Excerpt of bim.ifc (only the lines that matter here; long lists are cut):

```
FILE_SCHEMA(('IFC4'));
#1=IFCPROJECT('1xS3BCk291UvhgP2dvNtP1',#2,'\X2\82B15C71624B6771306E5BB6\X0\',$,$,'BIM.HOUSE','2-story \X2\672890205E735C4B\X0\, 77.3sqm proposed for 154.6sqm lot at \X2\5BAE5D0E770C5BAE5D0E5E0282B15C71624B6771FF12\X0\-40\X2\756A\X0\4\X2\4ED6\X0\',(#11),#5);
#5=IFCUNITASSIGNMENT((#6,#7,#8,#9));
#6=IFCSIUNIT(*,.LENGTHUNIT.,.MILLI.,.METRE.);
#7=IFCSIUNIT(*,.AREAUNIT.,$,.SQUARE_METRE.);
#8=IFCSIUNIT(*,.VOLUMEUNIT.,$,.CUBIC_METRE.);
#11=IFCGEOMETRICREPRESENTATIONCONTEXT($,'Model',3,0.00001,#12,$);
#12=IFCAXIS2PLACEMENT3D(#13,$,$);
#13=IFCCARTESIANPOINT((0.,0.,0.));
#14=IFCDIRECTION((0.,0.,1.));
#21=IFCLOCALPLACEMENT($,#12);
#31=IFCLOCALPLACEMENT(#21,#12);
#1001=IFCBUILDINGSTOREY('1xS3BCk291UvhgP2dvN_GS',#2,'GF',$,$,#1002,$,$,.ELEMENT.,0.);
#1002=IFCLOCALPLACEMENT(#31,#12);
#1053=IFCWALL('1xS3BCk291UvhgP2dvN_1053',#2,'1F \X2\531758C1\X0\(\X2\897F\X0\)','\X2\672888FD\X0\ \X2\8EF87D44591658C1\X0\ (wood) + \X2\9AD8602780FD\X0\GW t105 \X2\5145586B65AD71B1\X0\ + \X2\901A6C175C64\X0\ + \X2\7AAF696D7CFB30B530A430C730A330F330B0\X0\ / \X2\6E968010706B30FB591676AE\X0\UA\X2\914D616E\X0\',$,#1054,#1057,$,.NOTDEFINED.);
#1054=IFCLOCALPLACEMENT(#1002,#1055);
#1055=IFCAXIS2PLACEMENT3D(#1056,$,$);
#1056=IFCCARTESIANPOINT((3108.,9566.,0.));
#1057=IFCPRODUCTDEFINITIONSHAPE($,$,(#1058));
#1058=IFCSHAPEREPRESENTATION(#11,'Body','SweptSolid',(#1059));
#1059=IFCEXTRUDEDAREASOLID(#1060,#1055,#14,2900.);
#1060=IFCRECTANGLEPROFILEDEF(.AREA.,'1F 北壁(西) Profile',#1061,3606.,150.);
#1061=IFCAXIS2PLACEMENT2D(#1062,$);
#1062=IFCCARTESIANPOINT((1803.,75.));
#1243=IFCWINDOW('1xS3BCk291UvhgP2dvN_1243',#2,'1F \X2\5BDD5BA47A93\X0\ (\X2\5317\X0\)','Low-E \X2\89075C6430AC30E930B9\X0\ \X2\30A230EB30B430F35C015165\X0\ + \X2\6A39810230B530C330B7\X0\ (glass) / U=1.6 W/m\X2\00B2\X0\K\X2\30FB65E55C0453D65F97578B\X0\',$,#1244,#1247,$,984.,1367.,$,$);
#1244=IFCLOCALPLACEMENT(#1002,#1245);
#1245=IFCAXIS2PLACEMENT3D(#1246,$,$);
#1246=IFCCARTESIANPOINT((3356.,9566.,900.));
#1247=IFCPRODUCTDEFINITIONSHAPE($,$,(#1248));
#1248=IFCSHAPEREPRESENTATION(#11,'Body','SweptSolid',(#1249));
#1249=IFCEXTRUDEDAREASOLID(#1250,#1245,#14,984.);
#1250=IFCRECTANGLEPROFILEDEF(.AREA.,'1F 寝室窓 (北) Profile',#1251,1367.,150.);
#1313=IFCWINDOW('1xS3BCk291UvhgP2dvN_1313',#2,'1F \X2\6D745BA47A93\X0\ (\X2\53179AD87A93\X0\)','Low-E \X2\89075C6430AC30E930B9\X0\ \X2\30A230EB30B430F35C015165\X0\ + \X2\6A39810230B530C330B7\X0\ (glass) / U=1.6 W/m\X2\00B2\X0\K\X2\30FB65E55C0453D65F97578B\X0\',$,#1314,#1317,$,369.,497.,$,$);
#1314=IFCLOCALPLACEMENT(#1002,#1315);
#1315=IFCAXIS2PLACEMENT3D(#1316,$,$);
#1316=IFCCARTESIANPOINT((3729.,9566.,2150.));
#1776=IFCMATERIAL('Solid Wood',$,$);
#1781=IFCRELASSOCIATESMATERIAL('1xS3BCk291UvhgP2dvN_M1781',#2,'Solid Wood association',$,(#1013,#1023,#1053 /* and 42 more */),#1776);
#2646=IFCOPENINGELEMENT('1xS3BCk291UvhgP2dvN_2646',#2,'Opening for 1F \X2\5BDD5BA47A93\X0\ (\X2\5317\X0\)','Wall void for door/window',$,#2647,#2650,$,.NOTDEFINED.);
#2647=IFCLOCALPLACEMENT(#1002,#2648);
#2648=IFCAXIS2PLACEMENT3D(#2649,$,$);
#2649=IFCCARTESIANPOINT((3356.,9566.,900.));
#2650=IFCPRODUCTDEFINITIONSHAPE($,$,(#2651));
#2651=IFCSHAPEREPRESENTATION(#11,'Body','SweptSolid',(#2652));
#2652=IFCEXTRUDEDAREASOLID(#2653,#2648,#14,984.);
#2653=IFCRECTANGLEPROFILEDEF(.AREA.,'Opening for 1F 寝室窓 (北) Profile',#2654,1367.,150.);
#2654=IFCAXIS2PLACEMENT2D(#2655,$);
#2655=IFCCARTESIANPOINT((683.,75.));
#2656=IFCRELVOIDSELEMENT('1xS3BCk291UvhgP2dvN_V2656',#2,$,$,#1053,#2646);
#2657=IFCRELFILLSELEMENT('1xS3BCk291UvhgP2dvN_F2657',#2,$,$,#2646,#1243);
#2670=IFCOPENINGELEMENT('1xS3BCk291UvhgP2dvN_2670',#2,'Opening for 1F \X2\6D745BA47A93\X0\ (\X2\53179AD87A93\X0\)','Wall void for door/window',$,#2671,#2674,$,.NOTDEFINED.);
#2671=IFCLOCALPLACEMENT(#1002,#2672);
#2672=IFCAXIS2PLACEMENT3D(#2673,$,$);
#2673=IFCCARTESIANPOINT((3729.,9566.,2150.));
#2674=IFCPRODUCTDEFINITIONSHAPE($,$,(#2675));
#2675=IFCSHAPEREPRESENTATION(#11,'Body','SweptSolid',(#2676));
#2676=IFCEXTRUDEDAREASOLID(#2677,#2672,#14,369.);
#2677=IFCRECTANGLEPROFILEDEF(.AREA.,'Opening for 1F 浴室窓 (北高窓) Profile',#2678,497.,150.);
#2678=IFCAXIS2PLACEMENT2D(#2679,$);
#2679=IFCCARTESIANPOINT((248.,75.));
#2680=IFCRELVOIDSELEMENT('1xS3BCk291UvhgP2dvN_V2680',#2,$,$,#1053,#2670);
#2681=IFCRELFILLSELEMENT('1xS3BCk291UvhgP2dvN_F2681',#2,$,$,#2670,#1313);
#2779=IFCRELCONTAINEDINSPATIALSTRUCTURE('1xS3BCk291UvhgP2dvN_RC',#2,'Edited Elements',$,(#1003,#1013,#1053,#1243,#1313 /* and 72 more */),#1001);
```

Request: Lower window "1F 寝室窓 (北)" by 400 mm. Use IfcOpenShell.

```python
import numpy as np
import ifcopenshell
import ifcopenshell.api.geometry
import ifcopenshell.util.placement
import ifcopenshell.util.unit

model = ifcopenshell.open("bim.ifc")
unit_scale = ifcopenshell.util.unit.calculate_unit_scale(model)

window = model.by_guid("1xS3BCk291UvhgP2dvN_1243")
opening = window.FillsVoids[0].RelatingOpeningElement
dz = -0.4 / unit_scale

shift = np.array([0.0, 0.0, dz])
# The window is not placed relative to its opening, so move both.
for product in (opening, window):
    matrix = ifcopenshell.util.placement.get_local_placement(product.ObjectPlacement)
    matrix[:3, 3] += shift
    ifcopenshell.api.geometry.edit_object_placement(model, product=product, matrix=matrix, is_si=False)

print(f"moved by {dz * unit_scale:+.3f} m")

model.write("bim_updated.ifc")
```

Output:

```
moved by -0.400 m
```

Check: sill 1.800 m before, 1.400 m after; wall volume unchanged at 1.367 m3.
